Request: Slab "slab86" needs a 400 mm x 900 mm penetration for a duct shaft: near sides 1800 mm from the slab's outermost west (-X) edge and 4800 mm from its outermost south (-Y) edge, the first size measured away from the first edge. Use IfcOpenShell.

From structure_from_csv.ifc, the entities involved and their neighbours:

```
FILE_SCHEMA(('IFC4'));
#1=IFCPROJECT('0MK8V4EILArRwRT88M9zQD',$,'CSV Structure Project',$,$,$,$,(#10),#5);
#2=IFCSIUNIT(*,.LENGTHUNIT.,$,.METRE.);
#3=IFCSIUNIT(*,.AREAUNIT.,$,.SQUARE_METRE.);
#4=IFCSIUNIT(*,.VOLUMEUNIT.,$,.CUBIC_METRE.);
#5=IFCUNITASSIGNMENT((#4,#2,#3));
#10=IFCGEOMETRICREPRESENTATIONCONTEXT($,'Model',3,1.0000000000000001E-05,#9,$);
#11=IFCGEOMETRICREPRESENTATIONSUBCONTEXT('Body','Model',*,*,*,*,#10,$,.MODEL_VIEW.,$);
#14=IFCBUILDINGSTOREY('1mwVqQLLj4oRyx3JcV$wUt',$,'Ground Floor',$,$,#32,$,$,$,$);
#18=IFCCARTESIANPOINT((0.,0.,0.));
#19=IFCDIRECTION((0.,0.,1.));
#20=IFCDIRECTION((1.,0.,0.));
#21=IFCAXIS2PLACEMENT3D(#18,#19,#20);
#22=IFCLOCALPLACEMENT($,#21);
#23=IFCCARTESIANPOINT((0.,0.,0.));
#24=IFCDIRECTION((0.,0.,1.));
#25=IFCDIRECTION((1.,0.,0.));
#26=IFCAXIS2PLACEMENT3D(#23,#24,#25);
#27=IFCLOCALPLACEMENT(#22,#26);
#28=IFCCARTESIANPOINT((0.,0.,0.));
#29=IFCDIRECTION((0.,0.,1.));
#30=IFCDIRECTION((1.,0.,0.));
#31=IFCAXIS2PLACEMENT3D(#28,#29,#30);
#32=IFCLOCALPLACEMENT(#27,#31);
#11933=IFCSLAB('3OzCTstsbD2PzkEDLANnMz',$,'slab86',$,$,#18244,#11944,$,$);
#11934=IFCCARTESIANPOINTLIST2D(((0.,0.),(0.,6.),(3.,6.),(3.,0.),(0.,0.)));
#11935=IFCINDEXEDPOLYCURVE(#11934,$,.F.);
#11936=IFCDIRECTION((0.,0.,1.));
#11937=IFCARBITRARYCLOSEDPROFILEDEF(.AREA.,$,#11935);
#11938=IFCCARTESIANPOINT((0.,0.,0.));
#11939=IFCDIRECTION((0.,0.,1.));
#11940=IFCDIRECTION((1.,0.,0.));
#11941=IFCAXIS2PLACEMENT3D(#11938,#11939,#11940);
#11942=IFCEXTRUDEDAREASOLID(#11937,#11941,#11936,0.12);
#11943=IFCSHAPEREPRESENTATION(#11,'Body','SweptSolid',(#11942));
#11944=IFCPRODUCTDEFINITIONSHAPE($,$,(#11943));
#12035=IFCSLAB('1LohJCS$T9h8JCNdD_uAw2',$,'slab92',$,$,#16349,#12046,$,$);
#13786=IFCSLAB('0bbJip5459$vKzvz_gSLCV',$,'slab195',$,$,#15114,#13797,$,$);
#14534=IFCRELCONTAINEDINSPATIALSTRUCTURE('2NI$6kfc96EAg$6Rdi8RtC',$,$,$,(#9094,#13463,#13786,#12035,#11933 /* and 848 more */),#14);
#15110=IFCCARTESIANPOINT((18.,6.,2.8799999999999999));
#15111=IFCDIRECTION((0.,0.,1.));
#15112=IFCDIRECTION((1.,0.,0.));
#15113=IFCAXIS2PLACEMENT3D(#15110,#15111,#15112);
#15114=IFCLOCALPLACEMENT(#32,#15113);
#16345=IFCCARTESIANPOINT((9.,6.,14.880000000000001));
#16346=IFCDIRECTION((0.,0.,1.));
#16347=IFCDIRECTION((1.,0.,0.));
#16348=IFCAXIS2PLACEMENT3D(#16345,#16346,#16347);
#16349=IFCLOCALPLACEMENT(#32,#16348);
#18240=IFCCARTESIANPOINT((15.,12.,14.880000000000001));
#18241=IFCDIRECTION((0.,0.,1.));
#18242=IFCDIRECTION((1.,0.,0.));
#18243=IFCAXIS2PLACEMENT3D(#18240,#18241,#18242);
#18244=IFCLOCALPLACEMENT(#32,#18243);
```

```python
import numpy as np
import ifcopenshell
import ifcopenshell.api.feature
import ifcopenshell.api.geometry
import ifcopenshell.api.root
import ifcopenshell.geom
import ifcopenshell.util.placement
import ifcopenshell.util.representation
import ifcopenshell.util.shape
import ifcopenshell.util.unit

model = ifcopenshell.open("structure_from_csv.ifc")
unit_scale = ifcopenshell.util.unit.calculate_unit_scale(model)
settings = ifcopenshell.geom.settings()


def volume(element):
    """Net volume in cubic metres, openings subtracted."""
    shape = ifcopenshell.geom.create_shape(settings, element)
    return ifcopenshell.util.shape.get_volume(shape.geometry)


slab = model.by_id(11933)
before = volume(slab)

# Extent in the slab's own axes, in metres. The edges named are its -X and -Y sides.
slab_shape = ifcopenshell.geom.create_shape(settings, slab)
vertices = ifcopenshell.util.shape.get_vertices(slab_shape.geometry)
x_min, y_min, bottom = vertices.min(axis=0)
top = vertices[:, 2].max()

opening = ifcopenshell.api.root.create_entity(model, ifc_class="IfcOpeningElement", name="Duct shaft opening", predefined_type="OPENING")
context = ifcopenshell.util.representation.get_context(model, "Model", "Body", "MODEL_VIEW")
width, depth = 0.4, 0.9
outline = [(0.0, 0.0), (width, 0.0), (width, depth), (0.0, depth), (0.0, 0.0)]
# Overshoot both faces by 50 mm so the cut is clean.
shape = ifcopenshell.api.geometry.add_slab_representation(
    model, context=context, depth=top - bottom + 0.1, polyline=outline
)
ifcopenshell.api.geometry.assign_representation(model, product=opening, representation=shape)

matrix = ifcopenshell.util.placement.get_local_placement(slab.ObjectPlacement)
matrix[:, 3] = matrix @ np.append(np.array([x_min + 1.8, y_min + 4.8, bottom - 0.05]) / unit_scale, 1.0)
ifcopenshell.api.geometry.edit_object_placement(model, product=opening, matrix=matrix, is_si=False)
ifcopenshell.api.feature.add_feature(model, feature=opening, element=slab)

after = volume(slab)

print(f"slab volume {before:.3f} -> {after:.3f} m3")

model.write("structure_from_csv_edited.ifc")
```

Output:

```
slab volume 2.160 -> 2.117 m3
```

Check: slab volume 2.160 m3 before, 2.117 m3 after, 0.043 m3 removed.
